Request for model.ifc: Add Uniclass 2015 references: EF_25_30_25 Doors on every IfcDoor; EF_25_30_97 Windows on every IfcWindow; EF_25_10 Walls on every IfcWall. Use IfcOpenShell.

First a look at what the model holds.

```python
import ifcopenshell

model = ifcopenshell.open("model.ifc")
print(model.schema)
print("classifications:", [c.Name for c in model.by_type("IfcClassification")])
for ifc_class in ("IfcDoor", "IfcRoof", "IfcStair", "IfcWall", "IfcWindow"):
    print(ifc_class, len(model.by_type(ifc_class)))
```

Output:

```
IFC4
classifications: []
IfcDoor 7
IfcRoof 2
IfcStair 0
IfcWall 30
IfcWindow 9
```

```python
import ifcopenshell
import ifcopenshell.api.classification

model = ifcopenshell.open("model.ifc")

system = ifcopenshell.api.classification.add_classification(model, classification="Uniclass 2015")

codes = {
    "IfcDoor": ("EF_25_30_25", "Doors"),
    "IfcWindow": ("EF_25_30_97", "Windows"),
    "IfcWall": ("EF_25_10", "Walls"),
}
for ifc_class, (code, name) in codes.items():
    products = model.by_type(ifc_class)
    ifcopenshell.api.classification.add_reference(
        model, products=products, classification=system, identification=code, name=name
    )
    print(code, len(products))

model.write("model_edited.ifc")
```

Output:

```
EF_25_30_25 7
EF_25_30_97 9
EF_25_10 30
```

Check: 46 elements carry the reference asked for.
